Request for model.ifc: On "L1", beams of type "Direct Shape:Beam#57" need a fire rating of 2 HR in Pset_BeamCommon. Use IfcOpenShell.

First a look at what the model holds.

```python
import ifcopenshell
import ifcopenshell.util.element

model = ifcopenshell.open("model.ifc")
print(model.schema)
storey = next(s for s in model.by_type("IfcBuildingStorey") if s.Name == "L1")
beams = [e for e in ifcopenshell.util.element.get_decomposition(storey) if e.is_a("IfcBeam")]
seen = {}
for e in beams:
    element_type = ifcopenshell.util.element.get_type(e)
    key = (element_type.Name if element_type != e and element_type else None, ifcopenshell.util.element.get_pset(e, "Pset_BeamCommon", "FireRating"))
    seen[key] = seen.get(key, 0) + 1
for (name, value), count in sorted(seen.items(), key=str):
    print(count, "x", name, "|", value)
```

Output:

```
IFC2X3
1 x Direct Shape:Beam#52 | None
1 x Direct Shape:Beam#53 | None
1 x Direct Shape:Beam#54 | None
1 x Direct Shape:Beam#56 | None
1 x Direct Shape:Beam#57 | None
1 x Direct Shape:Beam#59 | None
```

```python
import ifcopenshell
import ifcopenshell.api.pset
import ifcopenshell.util.element

model = ifcopenshell.open("model.ifc")

storey = next(s for s in model.by_type("IfcBuildingStorey") if s.Name == "L1")
beams = [e for e in ifcopenshell.util.element.get_decomposition(storey) if e.is_a("IfcBeam")]

count = 0
for e in beams:
    element_type = ifcopenshell.util.element.get_type(e)
    if element_type in (None, e) or element_type.Name != "Direct Shape:Beam#57":
        continue
    # add_pset returns the element's existing set when there is one.
    pset = ifcopenshell.api.pset.add_pset(model, product=e, name="Pset_BeamCommon")
    ifcopenshell.api.pset.edit_pset(model, pset=pset, properties={"FireRating": "2 HR"})
    count += 1

print(count, "beams updated")

model.write("model-out.ifc")
```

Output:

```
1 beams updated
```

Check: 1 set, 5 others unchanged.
